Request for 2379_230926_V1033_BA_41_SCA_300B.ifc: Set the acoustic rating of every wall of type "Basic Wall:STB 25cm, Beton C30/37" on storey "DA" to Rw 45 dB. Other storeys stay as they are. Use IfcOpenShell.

First a look at what the model holds.

```python
import ifcopenshell
import ifcopenshell.util.element

model = ifcopenshell.open("2379_230926_V1033_BA_41_SCA_300B.ifc")
print(model.schema)
storey = next(s for s in model.by_type("IfcBuildingStorey") if s.Name == "DA")
walls = [e for e in ifcopenshell.util.element.get_decomposition(storey) if e.is_a("IfcWall")]
seen = {}
for e in walls:
    element_type = ifcopenshell.util.element.get_type(e)
    key = (element_type.Name if element_type != e and element_type else None, ifcopenshell.util.element.get_pset(e, "Pset_WallCommon", "AcousticRating"))
    seen[key] = seen.get(key, 0) + 1
for (name, value), count in sorted(seen.items(), key=str):
    print(count, "x", name, "|", value)
```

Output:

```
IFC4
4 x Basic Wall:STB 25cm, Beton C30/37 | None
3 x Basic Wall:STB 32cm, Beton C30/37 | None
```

```python
import ifcopenshell
import ifcopenshell.api.pset
import ifcopenshell.util.element

model = ifcopenshell.open("2379_230926_V1033_BA_41_SCA_300B.ifc")

storey = next(s for s in model.by_type("IfcBuildingStorey") if s.Name == "DA")
walls = [e for e in ifcopenshell.util.element.get_decomposition(storey) if e.is_a("IfcWall")]

count = 0
for e in walls:
    element_type = ifcopenshell.util.element.get_type(e)
    if element_type in (None, e) or element_type.Name != "Basic Wall:STB 25cm, Beton C30/37":
        continue
    # add_pset returns the element's existing set when there is one.
    pset = ifcopenshell.api.pset.add_pset(model, product=e, name="Pset_WallCommon")
    ifcopenshell.api.pset.edit_pset(model, pset=pset, properties={"AcousticRating": "Rw 45 dB"})
    count += 1

print(count, "walls updated")

model.write("2379_230926_V1033_BA_41_SCA_300B_rev.ifc")
```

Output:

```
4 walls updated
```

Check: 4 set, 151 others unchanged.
